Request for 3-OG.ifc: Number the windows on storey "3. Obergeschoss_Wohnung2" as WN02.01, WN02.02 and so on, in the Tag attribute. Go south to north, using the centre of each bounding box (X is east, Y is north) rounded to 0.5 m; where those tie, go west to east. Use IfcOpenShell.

First a look at what the model holds.

```python
import ifcopenshell
import ifcopenshell.util.element
import ifcopenshell.util.placement

model = ifcopenshell.open("3-OG.ifc")
print(model.schema)
storey = next(s for s in model.by_type("IfcBuildingStorey") if s.Name == "3. Obergeschoss_Wohnung2")
windows = [e for e in ifcopenshell.util.element.get_decomposition(storey) if e.is_a("IfcWindow")]
for e in sorted(windows, key=lambda e: e.id()):
    origin = ifcopenshell.util.placement.get_local_placement(e.ObjectPlacement)[:3, 3]
    print(e.id(), e.Tag, e.Name, origin.round(2) + 0.0, sep=" | ")
```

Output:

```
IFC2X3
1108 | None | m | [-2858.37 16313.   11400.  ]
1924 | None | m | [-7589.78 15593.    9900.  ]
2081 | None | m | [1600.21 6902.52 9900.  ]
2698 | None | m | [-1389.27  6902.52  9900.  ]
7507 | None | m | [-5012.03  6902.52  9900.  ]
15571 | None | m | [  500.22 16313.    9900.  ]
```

```python
import ifcopenshell
import ifcopenshell.geom
import ifcopenshell.util.element
import ifcopenshell.util.shape

model = ifcopenshell.open("3-OG.ifc")
settings = ifcopenshell.geom.settings()
settings.set("use-world-coords", True)


def centre(element):
    shape = ifcopenshell.geom.create_shape(settings, element)
    return ifcopenshell.util.shape.get_bbox_centroid(shape.geometry)


storey = next(s for s in model.by_type("IfcBuildingStorey") if s.Name == "3. Obergeschoss_Wohnung2")
windows = [e for e in ifcopenshell.util.element.get_decomposition(storey) if e.is_a("IfcWindow")]

# Insertion points can sit at a corner or the storey origin, so sort by the geometry (in metres).
centres = {e: centre(e) for e in windows}
windows.sort(key=lambda e: (round(centres[e][1] / 0.5), centres[e][0]))

for i, e in enumerate(windows, start=1):
    number = f"WN02.{i:02d}"
    e.Tag = number
    print(e.id(), number)

model.write("3-OG_v2.ifc")
```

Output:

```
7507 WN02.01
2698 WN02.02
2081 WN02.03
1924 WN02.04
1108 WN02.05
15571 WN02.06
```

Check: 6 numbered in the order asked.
